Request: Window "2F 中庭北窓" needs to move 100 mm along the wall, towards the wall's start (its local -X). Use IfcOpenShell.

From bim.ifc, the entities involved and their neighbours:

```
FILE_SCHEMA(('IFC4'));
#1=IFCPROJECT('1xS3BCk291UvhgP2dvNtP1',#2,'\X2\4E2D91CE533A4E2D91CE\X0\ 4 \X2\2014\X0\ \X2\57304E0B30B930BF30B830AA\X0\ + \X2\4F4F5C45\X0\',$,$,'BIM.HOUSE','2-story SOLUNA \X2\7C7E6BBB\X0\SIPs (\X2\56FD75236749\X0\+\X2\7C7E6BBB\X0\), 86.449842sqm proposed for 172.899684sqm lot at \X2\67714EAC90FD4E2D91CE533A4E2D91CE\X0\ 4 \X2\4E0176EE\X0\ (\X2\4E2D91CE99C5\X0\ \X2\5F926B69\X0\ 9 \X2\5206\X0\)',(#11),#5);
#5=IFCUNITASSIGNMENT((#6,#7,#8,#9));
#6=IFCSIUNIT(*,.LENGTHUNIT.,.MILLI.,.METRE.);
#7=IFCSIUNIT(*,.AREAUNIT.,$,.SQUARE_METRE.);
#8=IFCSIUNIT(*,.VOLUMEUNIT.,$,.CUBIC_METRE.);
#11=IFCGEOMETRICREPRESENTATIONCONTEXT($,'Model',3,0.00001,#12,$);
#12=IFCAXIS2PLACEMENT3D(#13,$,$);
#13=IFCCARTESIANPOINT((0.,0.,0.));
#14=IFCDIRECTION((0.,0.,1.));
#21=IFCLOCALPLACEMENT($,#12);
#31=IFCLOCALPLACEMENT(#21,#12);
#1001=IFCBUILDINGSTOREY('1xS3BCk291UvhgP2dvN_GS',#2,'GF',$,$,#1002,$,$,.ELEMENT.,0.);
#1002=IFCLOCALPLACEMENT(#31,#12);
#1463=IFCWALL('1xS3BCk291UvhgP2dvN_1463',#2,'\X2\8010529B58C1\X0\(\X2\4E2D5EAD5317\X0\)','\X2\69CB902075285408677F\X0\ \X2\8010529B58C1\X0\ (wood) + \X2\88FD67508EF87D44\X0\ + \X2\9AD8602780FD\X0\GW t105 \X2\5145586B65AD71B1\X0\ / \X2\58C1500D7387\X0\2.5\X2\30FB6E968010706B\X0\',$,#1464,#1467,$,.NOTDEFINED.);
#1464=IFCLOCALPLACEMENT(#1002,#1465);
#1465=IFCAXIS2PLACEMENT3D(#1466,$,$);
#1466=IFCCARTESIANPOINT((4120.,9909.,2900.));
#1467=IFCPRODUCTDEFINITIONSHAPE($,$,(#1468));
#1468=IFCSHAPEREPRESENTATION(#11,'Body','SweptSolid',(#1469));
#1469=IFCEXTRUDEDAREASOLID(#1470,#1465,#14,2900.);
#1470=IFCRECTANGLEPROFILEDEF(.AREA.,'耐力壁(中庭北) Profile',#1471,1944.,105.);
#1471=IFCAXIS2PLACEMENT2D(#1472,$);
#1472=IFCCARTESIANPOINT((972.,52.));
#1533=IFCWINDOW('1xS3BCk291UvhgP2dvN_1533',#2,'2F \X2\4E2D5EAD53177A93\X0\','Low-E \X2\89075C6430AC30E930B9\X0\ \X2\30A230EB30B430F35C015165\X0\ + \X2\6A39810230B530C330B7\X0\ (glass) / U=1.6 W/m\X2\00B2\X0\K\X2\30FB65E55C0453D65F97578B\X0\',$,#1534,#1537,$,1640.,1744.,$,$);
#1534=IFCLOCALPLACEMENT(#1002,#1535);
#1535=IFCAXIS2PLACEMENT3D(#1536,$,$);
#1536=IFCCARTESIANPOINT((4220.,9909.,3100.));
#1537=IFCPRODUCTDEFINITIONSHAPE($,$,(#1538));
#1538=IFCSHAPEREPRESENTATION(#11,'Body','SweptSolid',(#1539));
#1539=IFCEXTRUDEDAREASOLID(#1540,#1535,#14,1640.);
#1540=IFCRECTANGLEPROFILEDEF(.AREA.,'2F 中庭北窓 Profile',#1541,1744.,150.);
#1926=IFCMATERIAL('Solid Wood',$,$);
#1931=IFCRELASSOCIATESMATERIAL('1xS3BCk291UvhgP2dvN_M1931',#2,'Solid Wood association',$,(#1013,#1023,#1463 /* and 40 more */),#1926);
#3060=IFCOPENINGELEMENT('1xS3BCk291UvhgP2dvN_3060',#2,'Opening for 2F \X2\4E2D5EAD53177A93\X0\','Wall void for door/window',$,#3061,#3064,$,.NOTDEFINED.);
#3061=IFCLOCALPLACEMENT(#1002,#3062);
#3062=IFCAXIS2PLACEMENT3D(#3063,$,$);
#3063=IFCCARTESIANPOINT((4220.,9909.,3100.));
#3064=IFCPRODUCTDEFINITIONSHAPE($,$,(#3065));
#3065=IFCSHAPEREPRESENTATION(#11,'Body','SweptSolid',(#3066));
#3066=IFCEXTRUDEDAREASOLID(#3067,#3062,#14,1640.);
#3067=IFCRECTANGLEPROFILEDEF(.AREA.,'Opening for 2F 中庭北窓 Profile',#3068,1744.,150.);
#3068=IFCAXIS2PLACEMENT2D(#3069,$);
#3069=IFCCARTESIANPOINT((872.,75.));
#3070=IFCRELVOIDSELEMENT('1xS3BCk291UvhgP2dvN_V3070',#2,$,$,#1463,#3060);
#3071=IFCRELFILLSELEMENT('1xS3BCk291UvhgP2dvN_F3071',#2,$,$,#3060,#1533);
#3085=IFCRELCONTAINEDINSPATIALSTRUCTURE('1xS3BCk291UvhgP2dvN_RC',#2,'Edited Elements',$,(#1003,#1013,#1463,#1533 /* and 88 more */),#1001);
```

```python
import ifcopenshell
import ifcopenshell.api.geometry
import ifcopenshell.util.placement

model = ifcopenshell.open("bim.ifc")

window = model.by_guid("1xS3BCk291UvhgP2dvN_1533")
opening = window.FillsVoids[0].RelatingOpeningElement
wall = opening.VoidsElements[0].RelatingBuildingElement

wall_matrix = ifcopenshell.util.placement.get_local_placement(wall.ObjectPlacement)
shift = wall_matrix[:3, 0] * -100.0
before = ifcopenshell.util.placement.get_local_placement(window.ObjectPlacement)[:3, 3].copy()

# The window is not placed relative to its opening, so move both.
for product in (opening, window):
    matrix = ifcopenshell.util.placement.get_local_placement(product.ObjectPlacement)
    matrix[:3, 3] += shift
    ifcopenshell.api.geometry.edit_object_placement(model, product=product, matrix=matrix, is_si=False)

after = ifcopenshell.util.placement.get_local_placement(window.ObjectPlacement)[:3, 3]
print("window moved by", (after - before).round(3) + 0.0)

model.write("bim-out.ifc")
```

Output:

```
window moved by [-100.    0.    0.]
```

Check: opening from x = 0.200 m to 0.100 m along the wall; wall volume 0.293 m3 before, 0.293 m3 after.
